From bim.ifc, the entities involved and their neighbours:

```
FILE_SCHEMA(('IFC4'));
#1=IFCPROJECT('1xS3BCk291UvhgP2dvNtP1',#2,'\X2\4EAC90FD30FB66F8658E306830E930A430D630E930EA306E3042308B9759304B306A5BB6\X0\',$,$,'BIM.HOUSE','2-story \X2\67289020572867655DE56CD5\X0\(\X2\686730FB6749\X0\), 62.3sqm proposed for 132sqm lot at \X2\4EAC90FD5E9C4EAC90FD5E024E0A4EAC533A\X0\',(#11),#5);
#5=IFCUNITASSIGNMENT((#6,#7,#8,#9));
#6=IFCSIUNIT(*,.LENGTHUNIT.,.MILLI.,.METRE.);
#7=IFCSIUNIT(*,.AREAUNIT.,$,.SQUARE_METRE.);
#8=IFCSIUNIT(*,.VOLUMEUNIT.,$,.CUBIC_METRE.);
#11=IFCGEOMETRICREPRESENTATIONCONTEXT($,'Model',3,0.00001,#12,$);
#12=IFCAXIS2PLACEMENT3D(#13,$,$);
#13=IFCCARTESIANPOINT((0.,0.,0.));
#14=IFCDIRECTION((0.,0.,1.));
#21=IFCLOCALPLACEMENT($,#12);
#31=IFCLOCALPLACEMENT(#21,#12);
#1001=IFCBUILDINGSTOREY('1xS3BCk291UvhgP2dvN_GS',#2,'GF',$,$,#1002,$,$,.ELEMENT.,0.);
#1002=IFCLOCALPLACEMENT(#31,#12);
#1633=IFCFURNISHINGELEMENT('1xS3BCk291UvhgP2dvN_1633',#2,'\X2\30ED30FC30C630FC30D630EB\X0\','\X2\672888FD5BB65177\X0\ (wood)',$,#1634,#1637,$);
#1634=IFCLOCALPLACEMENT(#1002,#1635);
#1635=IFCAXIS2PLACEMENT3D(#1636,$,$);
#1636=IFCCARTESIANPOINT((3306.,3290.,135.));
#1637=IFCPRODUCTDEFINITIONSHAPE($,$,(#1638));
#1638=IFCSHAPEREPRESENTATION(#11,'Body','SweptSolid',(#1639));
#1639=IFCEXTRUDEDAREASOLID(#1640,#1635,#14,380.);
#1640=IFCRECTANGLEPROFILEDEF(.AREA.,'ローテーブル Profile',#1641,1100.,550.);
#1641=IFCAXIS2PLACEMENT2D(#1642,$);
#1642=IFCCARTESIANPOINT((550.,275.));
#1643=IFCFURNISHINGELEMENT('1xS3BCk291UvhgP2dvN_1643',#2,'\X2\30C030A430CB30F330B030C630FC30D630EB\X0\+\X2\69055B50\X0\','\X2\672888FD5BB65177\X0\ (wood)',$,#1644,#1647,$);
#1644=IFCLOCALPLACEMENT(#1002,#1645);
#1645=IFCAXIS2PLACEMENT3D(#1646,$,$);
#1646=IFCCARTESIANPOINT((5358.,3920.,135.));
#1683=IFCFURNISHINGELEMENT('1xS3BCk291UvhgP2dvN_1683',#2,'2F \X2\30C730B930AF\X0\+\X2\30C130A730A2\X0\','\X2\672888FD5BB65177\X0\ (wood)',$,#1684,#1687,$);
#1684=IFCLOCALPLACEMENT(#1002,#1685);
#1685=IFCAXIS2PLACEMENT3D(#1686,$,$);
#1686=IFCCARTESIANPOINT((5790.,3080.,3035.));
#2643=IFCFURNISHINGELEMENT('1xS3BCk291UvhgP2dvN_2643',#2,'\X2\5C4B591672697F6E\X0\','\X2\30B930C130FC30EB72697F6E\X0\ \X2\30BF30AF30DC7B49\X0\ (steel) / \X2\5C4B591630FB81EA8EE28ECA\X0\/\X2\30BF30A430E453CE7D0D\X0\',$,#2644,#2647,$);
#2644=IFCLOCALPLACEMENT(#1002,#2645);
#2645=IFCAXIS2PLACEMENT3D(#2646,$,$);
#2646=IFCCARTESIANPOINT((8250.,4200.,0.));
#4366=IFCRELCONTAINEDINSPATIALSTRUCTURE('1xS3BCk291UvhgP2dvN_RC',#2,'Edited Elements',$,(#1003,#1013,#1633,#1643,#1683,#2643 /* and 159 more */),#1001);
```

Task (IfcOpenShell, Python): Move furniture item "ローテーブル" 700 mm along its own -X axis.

```python
import ifcopenshell
import ifcopenshell.api.geometry
import ifcopenshell.util.placement

model = ifcopenshell.open("bim.ifc")

item = model.by_guid("1xS3BCk291UvhgP2dvN_1633")
matrix = ifcopenshell.util.placement.get_local_placement(item.ObjectPlacement)
matrix[:3, 3] -= matrix[:3, 0] * 700.0
ifcopenshell.api.geometry.edit_object_placement(model, product=item, matrix=matrix, is_si=False)

print(ifcopenshell.util.placement.get_local_placement(item.ObjectPlacement).round(3) + 0.0)

model.write("bim-out.ifc")
```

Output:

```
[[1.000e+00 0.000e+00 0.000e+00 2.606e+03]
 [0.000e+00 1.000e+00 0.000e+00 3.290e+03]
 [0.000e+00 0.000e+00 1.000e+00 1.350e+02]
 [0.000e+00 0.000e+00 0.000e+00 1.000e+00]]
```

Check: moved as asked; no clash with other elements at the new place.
